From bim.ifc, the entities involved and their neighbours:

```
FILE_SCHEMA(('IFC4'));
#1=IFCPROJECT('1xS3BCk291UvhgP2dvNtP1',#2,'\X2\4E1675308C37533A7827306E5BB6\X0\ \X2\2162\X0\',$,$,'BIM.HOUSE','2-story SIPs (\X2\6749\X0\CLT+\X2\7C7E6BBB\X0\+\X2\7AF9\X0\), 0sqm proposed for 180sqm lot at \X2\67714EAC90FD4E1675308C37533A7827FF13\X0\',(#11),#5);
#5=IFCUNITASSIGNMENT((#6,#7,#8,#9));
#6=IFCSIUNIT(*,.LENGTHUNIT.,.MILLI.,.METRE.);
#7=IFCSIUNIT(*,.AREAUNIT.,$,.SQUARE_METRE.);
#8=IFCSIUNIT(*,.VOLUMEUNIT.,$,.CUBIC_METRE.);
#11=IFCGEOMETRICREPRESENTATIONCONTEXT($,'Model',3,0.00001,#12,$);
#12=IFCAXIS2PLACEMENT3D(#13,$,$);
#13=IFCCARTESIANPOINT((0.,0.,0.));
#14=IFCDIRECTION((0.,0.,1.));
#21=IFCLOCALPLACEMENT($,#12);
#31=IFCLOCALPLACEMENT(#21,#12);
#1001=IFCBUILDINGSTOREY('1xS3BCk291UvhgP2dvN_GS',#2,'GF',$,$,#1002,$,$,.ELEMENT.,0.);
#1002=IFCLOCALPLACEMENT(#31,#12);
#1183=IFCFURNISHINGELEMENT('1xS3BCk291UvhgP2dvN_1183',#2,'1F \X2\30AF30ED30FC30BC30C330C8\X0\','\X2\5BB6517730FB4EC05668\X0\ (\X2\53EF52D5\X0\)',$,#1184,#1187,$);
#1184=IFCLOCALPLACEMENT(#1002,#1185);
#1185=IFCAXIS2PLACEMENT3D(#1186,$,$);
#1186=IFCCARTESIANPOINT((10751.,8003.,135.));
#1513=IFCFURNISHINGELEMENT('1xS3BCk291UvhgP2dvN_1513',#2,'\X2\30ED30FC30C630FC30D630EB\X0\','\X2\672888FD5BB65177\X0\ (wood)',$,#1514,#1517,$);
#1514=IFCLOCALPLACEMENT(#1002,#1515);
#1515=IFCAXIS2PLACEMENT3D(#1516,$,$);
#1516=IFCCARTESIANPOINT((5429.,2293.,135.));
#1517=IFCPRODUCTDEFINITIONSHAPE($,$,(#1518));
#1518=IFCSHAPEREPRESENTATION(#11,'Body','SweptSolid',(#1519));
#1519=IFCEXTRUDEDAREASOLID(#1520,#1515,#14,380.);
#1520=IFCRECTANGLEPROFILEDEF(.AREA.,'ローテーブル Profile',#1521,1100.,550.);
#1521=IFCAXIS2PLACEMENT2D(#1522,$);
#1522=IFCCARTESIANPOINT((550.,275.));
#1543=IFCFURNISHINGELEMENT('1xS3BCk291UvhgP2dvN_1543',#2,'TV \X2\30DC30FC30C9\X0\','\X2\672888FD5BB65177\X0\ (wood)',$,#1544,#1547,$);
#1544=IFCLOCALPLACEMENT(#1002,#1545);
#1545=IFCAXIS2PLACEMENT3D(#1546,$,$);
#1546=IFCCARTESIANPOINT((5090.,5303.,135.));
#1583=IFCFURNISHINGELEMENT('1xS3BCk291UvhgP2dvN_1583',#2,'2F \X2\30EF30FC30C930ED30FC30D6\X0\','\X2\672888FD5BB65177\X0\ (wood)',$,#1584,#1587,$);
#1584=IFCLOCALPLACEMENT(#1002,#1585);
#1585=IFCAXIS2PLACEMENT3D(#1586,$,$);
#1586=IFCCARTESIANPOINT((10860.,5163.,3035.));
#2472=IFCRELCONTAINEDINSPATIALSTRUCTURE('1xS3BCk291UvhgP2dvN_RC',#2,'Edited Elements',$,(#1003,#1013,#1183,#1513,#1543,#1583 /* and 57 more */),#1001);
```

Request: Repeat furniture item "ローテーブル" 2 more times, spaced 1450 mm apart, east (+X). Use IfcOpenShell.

```python
import numpy as np
import ifcopenshell
import ifcopenshell.api.geometry
import ifcopenshell.api.root
import ifcopenshell.util.element
import ifcopenshell.util.placement
import ifcopenshell.util.unit

model = ifcopenshell.open("bim.ifc")
unit_scale = ifcopenshell.util.unit.calculate_unit_scale(model)


def reuse_history(source, copy):
    """copy_class also copies each property set's owner history, people and application; keep the originals."""
    for rel in copy.IsDefinedBy:
        if rel.is_a("IfcRelDefinesByProperties") and (history := rel.RelatingPropertyDefinition.OwnerHistory):
            rel.RelatingPropertyDefinition.OwnerHistory = source.OwnerHistory
            ifcopenshell.util.element.remove_deep2(model, history)


source = model.by_id(1513)
base = ifcopenshell.util.placement.get_local_placement(source.ObjectPlacement)
step = np.array([1.0, 0.0, 0.0]) * 1.45 / unit_scale

for i in range(1, 3):
    copy = ifcopenshell.api.root.copy_class(model, product=source)
    copy.Representation = ifcopenshell.util.element.copy_deep(
        model, source.Representation, exclude=["IfcGeometricRepresentationContext", "IfcRepresentationMap"]
    )
    reuse_history(source, copy)
    matrix = base.copy()
    matrix[:3, 3] += i * step
    print("added at", matrix[:3, 3].round(3) + 0.0)
    ifcopenshell.api.geometry.edit_object_placement(model, product=copy, matrix=matrix, is_si=False)

model.write("bim_updated.ifc")
```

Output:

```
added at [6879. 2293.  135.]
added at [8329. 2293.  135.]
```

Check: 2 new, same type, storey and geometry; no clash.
